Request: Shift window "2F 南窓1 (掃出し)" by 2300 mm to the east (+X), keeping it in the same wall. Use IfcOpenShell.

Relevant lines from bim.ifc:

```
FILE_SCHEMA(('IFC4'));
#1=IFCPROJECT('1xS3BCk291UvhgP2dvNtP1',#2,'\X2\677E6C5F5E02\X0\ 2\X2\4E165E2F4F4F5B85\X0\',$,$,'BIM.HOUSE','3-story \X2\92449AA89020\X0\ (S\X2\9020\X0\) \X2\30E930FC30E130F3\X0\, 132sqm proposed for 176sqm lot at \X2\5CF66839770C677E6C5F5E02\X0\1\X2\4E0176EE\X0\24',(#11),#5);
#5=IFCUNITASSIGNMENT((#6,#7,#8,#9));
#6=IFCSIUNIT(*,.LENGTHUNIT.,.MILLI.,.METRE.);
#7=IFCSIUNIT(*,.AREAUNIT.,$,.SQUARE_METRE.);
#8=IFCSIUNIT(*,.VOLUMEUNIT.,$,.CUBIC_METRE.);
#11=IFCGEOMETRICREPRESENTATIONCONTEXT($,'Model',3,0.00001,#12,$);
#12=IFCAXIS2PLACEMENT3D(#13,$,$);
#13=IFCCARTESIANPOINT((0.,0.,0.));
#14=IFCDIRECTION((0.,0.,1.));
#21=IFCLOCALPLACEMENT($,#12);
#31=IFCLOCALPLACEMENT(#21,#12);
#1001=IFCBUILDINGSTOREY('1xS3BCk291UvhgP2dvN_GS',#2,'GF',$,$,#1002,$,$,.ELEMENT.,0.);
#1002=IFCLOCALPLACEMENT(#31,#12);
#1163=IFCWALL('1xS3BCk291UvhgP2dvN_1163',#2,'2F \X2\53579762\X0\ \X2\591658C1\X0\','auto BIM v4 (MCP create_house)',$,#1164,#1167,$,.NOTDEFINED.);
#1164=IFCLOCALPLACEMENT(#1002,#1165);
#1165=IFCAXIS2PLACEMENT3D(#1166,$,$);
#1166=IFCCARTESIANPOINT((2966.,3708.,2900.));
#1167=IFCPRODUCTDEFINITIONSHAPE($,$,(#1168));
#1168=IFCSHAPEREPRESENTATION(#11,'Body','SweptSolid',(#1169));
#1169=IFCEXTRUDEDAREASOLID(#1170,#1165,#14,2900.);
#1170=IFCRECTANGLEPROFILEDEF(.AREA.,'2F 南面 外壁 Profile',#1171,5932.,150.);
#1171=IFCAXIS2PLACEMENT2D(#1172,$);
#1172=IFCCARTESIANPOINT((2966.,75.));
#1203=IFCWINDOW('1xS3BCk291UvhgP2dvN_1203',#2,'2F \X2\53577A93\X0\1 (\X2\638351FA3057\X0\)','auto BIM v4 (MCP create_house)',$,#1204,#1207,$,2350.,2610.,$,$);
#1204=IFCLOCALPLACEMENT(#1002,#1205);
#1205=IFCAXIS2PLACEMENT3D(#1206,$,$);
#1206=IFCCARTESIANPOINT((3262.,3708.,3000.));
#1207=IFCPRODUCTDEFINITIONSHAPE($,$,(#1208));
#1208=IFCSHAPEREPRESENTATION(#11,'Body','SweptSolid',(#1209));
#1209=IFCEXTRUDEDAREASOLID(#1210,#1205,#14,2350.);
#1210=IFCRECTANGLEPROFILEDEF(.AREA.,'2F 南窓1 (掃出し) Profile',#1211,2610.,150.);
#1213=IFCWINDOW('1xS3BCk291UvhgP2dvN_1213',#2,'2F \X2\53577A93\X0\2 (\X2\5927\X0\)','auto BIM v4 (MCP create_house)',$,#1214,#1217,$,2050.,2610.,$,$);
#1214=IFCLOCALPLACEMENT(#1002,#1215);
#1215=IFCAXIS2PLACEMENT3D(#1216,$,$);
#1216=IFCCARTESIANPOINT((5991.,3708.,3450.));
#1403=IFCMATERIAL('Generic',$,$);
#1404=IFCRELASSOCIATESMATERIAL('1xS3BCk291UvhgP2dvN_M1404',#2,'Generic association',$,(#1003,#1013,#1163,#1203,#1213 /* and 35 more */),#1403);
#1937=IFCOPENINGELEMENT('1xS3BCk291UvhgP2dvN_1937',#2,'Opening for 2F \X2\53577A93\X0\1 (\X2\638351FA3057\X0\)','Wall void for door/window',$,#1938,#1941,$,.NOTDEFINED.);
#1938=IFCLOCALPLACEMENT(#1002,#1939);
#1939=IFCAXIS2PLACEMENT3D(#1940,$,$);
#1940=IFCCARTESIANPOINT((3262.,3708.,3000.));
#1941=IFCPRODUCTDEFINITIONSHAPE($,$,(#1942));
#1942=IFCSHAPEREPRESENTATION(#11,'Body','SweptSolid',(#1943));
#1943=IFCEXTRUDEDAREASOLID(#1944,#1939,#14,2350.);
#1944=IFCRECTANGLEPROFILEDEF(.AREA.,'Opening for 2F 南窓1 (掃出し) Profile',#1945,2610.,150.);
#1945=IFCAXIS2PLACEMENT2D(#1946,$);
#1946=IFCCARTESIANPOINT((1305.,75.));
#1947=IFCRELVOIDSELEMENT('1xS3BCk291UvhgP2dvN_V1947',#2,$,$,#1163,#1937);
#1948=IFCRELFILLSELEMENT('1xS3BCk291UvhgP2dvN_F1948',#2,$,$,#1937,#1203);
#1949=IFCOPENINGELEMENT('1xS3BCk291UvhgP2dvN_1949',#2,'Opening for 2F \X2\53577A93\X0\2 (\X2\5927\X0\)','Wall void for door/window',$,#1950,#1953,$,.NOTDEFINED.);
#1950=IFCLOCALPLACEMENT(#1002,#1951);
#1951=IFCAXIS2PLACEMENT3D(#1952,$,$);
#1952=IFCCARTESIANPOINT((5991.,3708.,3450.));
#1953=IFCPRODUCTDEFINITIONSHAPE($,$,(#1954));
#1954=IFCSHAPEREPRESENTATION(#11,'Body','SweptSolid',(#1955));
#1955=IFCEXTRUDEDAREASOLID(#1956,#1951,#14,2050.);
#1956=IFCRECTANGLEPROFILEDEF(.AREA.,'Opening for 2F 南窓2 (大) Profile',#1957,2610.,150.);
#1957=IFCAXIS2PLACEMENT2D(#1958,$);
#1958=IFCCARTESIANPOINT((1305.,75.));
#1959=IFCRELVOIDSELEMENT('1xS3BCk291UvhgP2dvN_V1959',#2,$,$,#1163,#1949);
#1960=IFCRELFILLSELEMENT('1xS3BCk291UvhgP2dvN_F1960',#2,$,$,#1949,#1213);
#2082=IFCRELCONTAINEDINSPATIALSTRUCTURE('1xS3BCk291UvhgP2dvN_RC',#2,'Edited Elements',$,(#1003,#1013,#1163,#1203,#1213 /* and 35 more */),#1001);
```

```python
import ifcopenshell
import ifcopenshell.api.geometry
import ifcopenshell.util.placement

model = ifcopenshell.open("bim.ifc")

window = model.by_guid("1xS3BCk291UvhgP2dvN_1203")
opening = window.FillsVoids[0].RelatingOpeningElement
wall = opening.VoidsElements[0].RelatingBuildingElement

wall_matrix = ifcopenshell.util.placement.get_local_placement(wall.ObjectPlacement)
shift = wall_matrix[:3, 0] * 2300.0
before = ifcopenshell.util.placement.get_local_placement(window.ObjectPlacement)[:3, 3].copy()

# The window is not placed relative to its opening, so move both.
for product in (opening, window):
    matrix = ifcopenshell.util.placement.get_local_placement(product.ObjectPlacement)
    matrix[:3, 3] += shift
    ifcopenshell.api.geometry.edit_object_placement(model, product=product, matrix=matrix, is_si=False)

after = ifcopenshell.util.placement.get_local_placement(window.ObjectPlacement)[:3, 3]
print("window moved by", (after - before).round(3) + 0.0)

model.write("bim_edited.ifc")
```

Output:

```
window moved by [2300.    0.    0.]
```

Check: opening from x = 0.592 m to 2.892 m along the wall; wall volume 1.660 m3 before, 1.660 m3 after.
